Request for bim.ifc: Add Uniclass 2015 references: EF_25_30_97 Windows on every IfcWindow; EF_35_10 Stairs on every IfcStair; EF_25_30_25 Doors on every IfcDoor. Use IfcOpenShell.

First a look at what the model holds.

```python
import ifcopenshell

model = ifcopenshell.open("bim.ifc")
print(model.schema)
print("classifications:", [c.Name for c in model.by_type("IfcClassification")])
for ifc_class in ("IfcDoor", "IfcRoof", "IfcStair", "IfcWall", "IfcWindow"):
    print(ifc_class, len(model.by_type(ifc_class)))
```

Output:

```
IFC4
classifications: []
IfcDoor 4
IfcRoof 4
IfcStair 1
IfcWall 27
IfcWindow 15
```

```python
import ifcopenshell
import ifcopenshell.api.classification

model = ifcopenshell.open("bim.ifc")

system = ifcopenshell.api.classification.add_classification(model, classification="Uniclass 2015")

codes = {
    "IfcWindow": ("EF_25_30_97", "Windows"),
    "IfcStair": ("EF_35_10", "Stairs"),
    "IfcDoor": ("EF_25_30_25", "Doors"),
}
for ifc_class, (code, name) in codes.items():
    products = model.by_type(ifc_class)
    ifcopenshell.api.classification.add_reference(
        model, products=products, classification=system, identification=code, name=name
    )
    print(code, len(products))

model.write("bim_v2.ifc")
```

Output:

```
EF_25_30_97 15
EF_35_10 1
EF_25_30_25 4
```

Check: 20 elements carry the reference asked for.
